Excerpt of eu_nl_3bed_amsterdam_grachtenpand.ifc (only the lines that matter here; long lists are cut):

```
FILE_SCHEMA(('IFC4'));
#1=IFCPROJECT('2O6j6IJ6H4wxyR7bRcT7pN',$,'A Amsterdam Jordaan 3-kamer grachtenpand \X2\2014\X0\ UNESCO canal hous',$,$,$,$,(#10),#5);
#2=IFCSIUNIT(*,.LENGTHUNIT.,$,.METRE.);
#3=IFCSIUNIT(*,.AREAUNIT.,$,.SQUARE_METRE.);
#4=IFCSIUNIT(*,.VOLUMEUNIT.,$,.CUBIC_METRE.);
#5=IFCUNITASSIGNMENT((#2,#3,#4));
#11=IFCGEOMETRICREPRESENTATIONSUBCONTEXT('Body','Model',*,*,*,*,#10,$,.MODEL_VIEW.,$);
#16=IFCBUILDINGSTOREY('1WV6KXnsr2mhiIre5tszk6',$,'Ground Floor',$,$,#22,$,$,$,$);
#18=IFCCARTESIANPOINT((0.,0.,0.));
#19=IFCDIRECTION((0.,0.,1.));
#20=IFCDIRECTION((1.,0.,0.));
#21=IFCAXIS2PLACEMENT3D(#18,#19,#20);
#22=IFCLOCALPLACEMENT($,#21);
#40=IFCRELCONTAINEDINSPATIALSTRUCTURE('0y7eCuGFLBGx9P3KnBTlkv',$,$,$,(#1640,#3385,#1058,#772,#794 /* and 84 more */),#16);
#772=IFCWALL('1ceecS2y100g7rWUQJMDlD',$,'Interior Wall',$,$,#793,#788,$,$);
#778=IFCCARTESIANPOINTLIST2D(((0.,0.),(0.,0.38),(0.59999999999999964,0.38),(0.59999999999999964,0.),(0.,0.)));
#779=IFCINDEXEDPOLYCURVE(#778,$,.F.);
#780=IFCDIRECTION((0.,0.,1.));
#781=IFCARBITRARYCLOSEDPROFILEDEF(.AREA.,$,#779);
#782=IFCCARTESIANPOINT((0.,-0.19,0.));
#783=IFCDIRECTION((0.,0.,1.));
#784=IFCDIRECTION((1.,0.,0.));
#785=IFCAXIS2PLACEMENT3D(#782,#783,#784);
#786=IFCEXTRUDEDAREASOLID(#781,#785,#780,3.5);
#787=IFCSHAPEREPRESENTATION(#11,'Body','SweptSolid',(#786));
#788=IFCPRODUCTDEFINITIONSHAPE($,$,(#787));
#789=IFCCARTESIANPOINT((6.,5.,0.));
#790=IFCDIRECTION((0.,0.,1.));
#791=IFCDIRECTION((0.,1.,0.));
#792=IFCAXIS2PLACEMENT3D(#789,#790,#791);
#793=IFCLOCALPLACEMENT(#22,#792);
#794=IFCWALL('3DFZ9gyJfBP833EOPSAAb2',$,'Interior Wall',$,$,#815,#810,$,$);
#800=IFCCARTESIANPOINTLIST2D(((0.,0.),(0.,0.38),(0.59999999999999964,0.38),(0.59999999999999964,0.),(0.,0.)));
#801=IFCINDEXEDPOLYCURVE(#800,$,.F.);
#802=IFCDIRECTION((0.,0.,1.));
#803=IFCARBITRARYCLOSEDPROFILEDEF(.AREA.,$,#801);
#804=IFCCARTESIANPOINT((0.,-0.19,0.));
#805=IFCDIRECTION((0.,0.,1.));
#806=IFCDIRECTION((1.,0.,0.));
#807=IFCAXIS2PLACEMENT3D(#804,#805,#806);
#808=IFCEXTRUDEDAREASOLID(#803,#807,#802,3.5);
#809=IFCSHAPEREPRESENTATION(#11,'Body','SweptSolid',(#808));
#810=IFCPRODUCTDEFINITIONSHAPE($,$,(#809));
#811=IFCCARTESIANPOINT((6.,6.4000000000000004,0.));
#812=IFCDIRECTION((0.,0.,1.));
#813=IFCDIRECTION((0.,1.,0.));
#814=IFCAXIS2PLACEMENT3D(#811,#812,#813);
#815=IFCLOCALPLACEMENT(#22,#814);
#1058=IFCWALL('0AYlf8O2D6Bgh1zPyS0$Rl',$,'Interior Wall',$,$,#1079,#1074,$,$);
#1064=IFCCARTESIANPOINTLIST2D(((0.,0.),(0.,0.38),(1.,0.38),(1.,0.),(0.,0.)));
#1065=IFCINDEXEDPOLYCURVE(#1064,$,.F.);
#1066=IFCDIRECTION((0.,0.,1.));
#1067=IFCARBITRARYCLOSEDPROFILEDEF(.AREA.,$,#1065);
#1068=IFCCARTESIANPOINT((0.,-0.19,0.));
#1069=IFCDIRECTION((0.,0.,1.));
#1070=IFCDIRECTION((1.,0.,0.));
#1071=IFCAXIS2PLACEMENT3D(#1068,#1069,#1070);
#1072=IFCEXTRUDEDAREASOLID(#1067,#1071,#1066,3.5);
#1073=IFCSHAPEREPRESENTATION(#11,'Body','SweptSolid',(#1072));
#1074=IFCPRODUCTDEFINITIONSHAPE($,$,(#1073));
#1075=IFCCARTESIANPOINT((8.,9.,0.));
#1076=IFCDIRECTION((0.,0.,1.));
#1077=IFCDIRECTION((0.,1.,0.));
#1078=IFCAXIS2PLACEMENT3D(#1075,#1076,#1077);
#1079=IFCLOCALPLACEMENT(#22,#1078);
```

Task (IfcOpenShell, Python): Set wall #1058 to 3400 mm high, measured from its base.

```python
import ifcopenshell
import ifcopenshell.geom
import ifcopenshell.util.representation
import ifcopenshell.util.shape

model = ifcopenshell.open("eu_nl_3bed_amsterdam_grachtenpand.ifc")
settings = ifcopenshell.geom.settings()


def volume(element):
    """Net volume in cubic metres, openings subtracted."""
    shape = ifcopenshell.geom.create_shape(settings, element)
    return ifcopenshell.util.shape.get_volume(shape.geometry)


wall = model.by_guid("0AYlf8O2D6Bgh1zPyS0$Rl")
before = volume(wall)

body = ifcopenshell.util.representation.get_representation(wall, "Model", "Body")
solid = body.Items[0]
old_height = solid.Depth
solid.Depth = 3.4
after = volume(wall)

print(f"height {old_height:g} -> {solid.Depth:g}, volume {before:.3f} -> {after:.3f} m3")

model.write("eu_nl_3bed_amsterdam_grachtenpand_edited.ifc")
```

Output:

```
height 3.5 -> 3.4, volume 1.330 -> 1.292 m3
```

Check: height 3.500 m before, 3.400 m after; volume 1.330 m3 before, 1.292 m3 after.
